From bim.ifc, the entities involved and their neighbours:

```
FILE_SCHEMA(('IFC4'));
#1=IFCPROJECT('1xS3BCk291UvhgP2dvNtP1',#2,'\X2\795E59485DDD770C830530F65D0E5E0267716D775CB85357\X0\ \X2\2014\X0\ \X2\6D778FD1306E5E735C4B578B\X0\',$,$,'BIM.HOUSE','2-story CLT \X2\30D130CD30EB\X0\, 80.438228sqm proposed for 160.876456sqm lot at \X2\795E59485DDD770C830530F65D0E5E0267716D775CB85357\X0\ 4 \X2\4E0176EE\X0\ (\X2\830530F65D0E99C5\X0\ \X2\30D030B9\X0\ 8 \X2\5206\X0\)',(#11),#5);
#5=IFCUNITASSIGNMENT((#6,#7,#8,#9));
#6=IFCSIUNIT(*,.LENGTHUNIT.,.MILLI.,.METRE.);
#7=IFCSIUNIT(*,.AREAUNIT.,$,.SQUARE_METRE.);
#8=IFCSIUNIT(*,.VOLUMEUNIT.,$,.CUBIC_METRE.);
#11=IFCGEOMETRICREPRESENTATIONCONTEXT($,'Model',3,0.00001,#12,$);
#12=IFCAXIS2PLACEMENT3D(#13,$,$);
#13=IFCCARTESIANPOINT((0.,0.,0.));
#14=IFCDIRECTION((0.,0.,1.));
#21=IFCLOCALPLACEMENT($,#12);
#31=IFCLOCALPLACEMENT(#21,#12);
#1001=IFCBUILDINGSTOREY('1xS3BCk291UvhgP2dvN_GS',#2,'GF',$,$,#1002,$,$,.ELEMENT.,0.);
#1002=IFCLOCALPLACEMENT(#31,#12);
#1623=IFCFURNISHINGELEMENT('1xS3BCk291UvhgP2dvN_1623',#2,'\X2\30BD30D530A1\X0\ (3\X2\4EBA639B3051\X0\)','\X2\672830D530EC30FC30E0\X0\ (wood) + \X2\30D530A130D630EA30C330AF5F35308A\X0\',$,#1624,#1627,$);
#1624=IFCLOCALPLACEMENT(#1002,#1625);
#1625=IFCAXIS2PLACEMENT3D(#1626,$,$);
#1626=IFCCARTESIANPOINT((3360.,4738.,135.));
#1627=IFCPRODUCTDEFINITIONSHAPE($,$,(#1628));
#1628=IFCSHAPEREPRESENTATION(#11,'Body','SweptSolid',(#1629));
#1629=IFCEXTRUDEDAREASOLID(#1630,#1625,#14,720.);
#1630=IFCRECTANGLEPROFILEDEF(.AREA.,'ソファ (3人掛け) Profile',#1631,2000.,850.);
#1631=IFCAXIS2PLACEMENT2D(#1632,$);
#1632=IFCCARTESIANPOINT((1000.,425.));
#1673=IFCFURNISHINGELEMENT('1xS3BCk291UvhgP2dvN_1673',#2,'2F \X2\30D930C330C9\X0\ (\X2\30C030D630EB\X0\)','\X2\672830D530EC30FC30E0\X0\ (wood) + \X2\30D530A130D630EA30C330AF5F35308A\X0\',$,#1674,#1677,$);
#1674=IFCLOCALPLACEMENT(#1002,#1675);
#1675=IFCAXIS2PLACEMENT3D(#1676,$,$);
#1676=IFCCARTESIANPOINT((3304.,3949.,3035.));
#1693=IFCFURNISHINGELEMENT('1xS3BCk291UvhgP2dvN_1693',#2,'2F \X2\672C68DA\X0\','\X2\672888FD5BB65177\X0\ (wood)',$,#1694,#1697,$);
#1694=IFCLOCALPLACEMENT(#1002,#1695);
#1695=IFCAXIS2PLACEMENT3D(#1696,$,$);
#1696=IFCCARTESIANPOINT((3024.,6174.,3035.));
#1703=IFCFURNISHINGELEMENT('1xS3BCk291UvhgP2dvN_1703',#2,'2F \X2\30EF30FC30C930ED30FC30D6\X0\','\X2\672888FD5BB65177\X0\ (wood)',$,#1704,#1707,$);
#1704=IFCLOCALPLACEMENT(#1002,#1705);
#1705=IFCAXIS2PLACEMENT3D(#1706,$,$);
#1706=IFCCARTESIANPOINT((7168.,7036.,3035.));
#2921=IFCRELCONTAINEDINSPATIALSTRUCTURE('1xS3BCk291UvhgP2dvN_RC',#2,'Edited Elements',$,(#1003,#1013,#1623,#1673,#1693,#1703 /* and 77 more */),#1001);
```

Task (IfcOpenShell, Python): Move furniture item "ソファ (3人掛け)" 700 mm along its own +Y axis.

```python
import ifcopenshell
import ifcopenshell.api.geometry
import ifcopenshell.util.placement

model = ifcopenshell.open("bim.ifc")

item = model.by_guid("1xS3BCk291UvhgP2dvN_1623")
matrix = ifcopenshell.util.placement.get_local_placement(item.ObjectPlacement)
matrix[:3, 3] += matrix[:3, 1] * 700.0
ifcopenshell.api.geometry.edit_object_placement(model, product=item, matrix=matrix, is_si=False)

print(ifcopenshell.util.placement.get_local_placement(item.ObjectPlacement).round(3) + 0.0)

model.write("bim_v2.ifc")
```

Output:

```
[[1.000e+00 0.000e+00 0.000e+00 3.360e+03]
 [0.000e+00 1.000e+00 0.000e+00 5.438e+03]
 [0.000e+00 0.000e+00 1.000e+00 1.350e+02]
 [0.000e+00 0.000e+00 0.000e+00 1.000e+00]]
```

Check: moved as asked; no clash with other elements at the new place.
